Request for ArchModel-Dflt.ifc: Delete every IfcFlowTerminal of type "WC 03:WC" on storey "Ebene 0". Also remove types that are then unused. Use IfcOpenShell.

First a look at what the model holds.

```python
import ifcopenshell
import ifcopenshell.util.element

model = ifcopenshell.open("ArchModel-Dflt.ifc")
print(model.schema)
storey = next(s for s in model.by_type("IfcBuildingStorey") if s.Name == "Ebene 0")
terminals = [e for e in ifcopenshell.util.element.get_decomposition(storey) if e.is_a("IfcFlowTerminal")]
seen = {}
for e in terminals:
    element_type = ifcopenshell.util.element.get_type(e)
    name = element_type.Name if element_type not in (None, e) else None
    seen[name] = seen.get(name, 0) + 1
for name, count in sorted(seen.items(), key=str):
    print(count, "x", name)
```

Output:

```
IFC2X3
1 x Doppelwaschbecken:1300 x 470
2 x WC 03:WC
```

```python
import ifcopenshell
import ifcopenshell.api.root
import ifcopenshell.util.element

model = ifcopenshell.open("ArchModel-Dflt.ifc")

storey = next(s for s in model.by_type("IfcBuildingStorey") if s.Name == "Ebene 0")
terminals = [e for e in ifcopenshell.util.element.get_decomposition(storey) if e.is_a("IfcFlowTerminal")]
targets = [e for e in terminals if (t := ifcopenshell.util.element.get_type(e)) not in (None, e) and t.Name == "WC 03:WC"]
types = {ifcopenshell.util.element.get_type(e) for e in targets} - {None, *targets}

for e in targets:
    ifcopenshell.api.root.remove_product(model, product=e)
print(len(targets), "removed")

unused = [t for t in types if not ifcopenshell.util.element.get_types(t)]
for t in unused:
    ifcopenshell.api.root.remove_product(model, product=t)
print(len(unused), "unused types removed")

model.write("ArchModel-Dflt_edited.ifc")
```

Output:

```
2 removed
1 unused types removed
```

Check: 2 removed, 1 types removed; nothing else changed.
